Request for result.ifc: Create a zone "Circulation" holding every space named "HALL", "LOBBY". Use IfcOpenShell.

First a look at what the model holds.

```python
import ifcopenshell

model = ifcopenshell.open("result.ifc")
print(model.schema)
seen = {}
for space in model.by_type("IfcSpace"):
    seen[space.Name] = seen.get(space.Name, 0) + 1
for name, count in sorted(seen.items(), key=str):
    print(count, "x", name)
print("zones:", [z.Name for z in model.by_type("IfcZone")][:20])
```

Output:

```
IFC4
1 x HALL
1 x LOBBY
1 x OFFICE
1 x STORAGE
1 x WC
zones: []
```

```python
import ifcopenshell
import ifcopenshell.api.group
import ifcopenshell.api.root

model = ifcopenshell.open("result.ifc")

names = {"HALL", "LOBBY"}
spaces = [s for s in model.by_type("IfcSpace") if s.Name in names]

zone = ifcopenshell.api.root.create_entity(model, ifc_class="IfcZone", name="Circulation")
ifcopenshell.api.group.assign_group(model, products=spaces, group=zone)
print(len(spaces), "spaces in", zone.Name)

model.write("result_edited.ifc")
```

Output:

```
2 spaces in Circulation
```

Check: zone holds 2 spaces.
